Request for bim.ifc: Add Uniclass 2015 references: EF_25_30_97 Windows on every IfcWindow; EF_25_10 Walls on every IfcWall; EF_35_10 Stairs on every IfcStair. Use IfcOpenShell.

First a look at what the model holds.

```python
import ifcopenshell

model = ifcopenshell.open("bim.ifc")
print(model.schema)
print("classifications:", [c.Name for c in model.by_type("IfcClassification")])
for ifc_class in ("IfcDoor", "IfcRoof", "IfcStair", "IfcWall", "IfcWindow"):
    print(ifc_class, len(model.by_type(ifc_class)))
```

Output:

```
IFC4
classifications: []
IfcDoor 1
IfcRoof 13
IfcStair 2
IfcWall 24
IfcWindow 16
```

```python
import ifcopenshell
import ifcopenshell.api.classification

model = ifcopenshell.open("bim.ifc")

system = ifcopenshell.api.classification.add_classification(model, classification="Uniclass 2015")

codes = {
    "IfcWindow": ("EF_25_30_97", "Windows"),
    "IfcWall": ("EF_25_10", "Walls"),
    "IfcStair": ("EF_35_10", "Stairs"),
}
for ifc_class, (code, name) in codes.items():
    products = model.by_type(ifc_class)
    ifcopenshell.api.classification.add_reference(
        model, products=products, classification=system, identification=code, name=name
    )
    print(code, len(products))

model.write("bim_edited.ifc")
```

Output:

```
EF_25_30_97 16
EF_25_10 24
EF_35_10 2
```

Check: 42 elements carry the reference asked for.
